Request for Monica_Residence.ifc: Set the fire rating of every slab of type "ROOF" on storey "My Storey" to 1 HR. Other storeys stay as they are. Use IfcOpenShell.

First a look at what the model holds.

```python
import ifcopenshell
import ifcopenshell.util.element

model = ifcopenshell.open("Monica_Residence.ifc")
print(model.schema)
storey = next(s for s in model.by_type("IfcBuildingStorey") if s.Name == "My Storey")
slabs = [e for e in ifcopenshell.util.element.get_decomposition(storey) if e.is_a("IfcSlab")]
seen = {}
for e in slabs:
    element_type = ifcopenshell.util.element.get_type(e)
    key = (element_type.Name if element_type != e and element_type else None, ifcopenshell.util.element.get_pset(e, "Pset_SlabCommon", "FireRating"))
    seen[key] = seen.get(key, 0) + 1
for (name, value), count in sorted(seen.items(), key=str):
    print(count, "x", name, "|", value)
```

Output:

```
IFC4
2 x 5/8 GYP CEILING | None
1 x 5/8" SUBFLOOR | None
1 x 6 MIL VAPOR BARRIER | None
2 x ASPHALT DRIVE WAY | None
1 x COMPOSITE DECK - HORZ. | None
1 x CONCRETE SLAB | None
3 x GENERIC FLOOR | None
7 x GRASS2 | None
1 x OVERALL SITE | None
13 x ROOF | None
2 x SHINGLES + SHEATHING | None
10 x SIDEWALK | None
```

```python
import ifcopenshell
import ifcopenshell.api.pset
import ifcopenshell.util.element

model = ifcopenshell.open("Monica_Residence.ifc")

storey = next(s for s in model.by_type("IfcBuildingStorey") if s.Name == "My Storey")
slabs = [e for e in ifcopenshell.util.element.get_decomposition(storey) if e.is_a("IfcSlab")]

count = 0
for e in slabs:
    element_type = ifcopenshell.util.element.get_type(e)
    if element_type in (None, e) or element_type.Name != "ROOF":
        continue
    # add_pset returns the element's existing set when there is one.
    pset = ifcopenshell.api.pset.add_pset(model, product=e, name="Pset_SlabCommon")
    ifcopenshell.api.pset.edit_pset(model, pset=pset, properties={"FireRating": "1 HR"})
    count += 1

print(count, "slabs updated")

model.write("Monica_Residence-out.ifc")
```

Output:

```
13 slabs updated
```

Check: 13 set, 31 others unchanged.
